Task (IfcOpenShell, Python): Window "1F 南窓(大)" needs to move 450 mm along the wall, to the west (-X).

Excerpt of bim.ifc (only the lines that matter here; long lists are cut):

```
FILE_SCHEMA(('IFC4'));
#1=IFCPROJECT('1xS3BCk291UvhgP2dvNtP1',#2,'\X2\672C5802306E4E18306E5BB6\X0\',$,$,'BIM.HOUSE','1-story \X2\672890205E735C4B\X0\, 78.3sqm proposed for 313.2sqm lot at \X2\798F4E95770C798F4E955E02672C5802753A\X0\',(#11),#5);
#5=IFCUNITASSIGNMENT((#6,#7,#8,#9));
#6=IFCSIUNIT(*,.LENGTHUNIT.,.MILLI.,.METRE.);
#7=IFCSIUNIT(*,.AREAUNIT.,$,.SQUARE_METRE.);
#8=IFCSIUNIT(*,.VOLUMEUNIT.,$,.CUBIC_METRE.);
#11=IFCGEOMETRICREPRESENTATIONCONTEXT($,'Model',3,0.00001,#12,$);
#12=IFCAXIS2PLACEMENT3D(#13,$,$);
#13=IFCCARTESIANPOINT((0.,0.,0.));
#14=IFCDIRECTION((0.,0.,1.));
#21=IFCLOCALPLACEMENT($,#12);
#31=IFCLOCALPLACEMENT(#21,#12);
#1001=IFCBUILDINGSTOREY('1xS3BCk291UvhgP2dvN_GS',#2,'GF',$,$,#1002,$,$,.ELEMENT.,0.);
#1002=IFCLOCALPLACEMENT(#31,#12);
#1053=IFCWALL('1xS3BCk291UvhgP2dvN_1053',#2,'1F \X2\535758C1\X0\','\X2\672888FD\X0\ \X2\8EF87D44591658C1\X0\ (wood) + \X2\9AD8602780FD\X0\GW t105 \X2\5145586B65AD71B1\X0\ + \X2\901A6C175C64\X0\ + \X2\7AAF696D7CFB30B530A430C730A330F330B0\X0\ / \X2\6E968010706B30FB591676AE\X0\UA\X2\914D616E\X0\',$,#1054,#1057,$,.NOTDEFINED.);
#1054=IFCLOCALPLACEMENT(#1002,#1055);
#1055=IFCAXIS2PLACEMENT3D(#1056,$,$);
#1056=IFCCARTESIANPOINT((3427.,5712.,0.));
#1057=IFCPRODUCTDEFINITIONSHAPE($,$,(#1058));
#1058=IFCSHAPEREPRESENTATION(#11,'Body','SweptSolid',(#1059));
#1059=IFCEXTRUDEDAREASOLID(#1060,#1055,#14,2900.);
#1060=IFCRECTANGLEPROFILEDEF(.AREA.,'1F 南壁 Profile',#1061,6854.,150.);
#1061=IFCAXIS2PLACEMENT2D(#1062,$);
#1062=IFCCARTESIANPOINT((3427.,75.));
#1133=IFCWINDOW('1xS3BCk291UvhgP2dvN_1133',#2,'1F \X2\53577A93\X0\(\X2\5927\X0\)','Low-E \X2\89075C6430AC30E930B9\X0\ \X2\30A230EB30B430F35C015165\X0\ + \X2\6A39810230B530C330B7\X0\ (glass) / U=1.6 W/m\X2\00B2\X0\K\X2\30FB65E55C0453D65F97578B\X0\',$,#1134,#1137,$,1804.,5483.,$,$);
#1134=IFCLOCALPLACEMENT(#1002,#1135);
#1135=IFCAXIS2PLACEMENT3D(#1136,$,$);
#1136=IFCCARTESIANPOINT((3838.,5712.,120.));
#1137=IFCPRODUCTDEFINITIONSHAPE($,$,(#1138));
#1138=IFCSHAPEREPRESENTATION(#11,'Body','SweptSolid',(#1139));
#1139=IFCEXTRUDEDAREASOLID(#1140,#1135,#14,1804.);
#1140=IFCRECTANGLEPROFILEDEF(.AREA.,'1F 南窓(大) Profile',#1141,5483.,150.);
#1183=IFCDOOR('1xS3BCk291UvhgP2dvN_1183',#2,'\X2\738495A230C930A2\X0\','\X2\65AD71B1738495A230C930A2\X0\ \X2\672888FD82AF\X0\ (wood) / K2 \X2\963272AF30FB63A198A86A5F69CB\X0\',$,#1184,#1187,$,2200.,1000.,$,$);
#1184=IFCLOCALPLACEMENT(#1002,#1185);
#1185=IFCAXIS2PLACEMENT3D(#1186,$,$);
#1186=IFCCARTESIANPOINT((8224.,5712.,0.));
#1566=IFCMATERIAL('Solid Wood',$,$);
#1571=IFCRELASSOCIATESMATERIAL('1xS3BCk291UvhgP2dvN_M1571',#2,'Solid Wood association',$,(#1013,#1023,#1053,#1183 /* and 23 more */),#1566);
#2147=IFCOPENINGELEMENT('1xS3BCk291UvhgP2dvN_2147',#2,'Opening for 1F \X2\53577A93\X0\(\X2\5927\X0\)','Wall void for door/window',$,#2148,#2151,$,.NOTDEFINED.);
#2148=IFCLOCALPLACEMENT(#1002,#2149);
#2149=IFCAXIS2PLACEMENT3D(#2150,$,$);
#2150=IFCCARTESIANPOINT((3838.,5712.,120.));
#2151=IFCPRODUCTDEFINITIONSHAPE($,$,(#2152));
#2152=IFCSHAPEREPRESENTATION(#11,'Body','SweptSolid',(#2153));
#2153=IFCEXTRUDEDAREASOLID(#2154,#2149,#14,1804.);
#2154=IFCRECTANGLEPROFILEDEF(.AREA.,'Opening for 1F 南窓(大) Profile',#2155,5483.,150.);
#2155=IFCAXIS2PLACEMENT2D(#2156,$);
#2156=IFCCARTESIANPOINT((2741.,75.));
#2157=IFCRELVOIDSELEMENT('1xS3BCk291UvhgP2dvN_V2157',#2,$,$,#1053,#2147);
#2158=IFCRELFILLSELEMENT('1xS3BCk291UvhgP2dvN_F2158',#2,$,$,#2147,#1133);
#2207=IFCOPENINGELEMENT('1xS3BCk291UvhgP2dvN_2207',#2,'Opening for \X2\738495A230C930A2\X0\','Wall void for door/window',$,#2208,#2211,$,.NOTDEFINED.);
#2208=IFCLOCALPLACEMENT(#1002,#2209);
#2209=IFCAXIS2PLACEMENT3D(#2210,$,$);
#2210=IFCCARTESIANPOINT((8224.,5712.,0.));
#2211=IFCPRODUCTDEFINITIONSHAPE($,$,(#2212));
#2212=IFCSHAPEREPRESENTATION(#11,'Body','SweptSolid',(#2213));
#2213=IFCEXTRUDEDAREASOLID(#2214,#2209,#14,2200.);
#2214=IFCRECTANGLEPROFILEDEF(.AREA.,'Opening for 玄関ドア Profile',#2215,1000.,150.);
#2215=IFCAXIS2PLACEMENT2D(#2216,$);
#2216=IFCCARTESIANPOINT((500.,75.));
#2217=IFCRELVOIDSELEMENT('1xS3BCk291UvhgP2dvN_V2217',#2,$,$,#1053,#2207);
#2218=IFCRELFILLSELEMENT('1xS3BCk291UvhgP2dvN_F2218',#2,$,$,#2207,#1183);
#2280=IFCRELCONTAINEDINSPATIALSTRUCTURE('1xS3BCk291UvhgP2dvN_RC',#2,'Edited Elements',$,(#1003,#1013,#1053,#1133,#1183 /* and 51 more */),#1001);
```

```python
import ifcopenshell
import ifcopenshell.api.geometry
import ifcopenshell.util.placement
import ifcopenshell.util.unit

model = ifcopenshell.open("bim.ifc")
unit_scale = ifcopenshell.util.unit.calculate_unit_scale(model)

window = model.by_guid("1xS3BCk291UvhgP2dvN_1133")
opening = window.FillsVoids[0].RelatingOpeningElement
wall = opening.VoidsElements[0].RelatingBuildingElement

wall_matrix = ifcopenshell.util.placement.get_local_placement(wall.ObjectPlacement)
shift = wall_matrix[:3, 0] * -0.45 / unit_scale
before = ifcopenshell.util.placement.get_local_placement(window.ObjectPlacement)[:3, 3].copy()

# The window is not placed relative to its opening, so move both.
for product in (opening, window):
    matrix = ifcopenshell.util.placement.get_local_placement(product.ObjectPlacement)
    matrix[:3, 3] += shift
    ifcopenshell.api.geometry.edit_object_placement(model, product=product, matrix=matrix, is_si=False)

after = ifcopenshell.util.placement.get_local_placement(window.ObjectPlacement)[:3, 3]
print("window moved by", (after - before).round(3) + 0.0)

model.write("bim_rev.ifc")
```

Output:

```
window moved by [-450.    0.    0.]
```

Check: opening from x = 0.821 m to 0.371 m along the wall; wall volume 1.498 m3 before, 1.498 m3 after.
